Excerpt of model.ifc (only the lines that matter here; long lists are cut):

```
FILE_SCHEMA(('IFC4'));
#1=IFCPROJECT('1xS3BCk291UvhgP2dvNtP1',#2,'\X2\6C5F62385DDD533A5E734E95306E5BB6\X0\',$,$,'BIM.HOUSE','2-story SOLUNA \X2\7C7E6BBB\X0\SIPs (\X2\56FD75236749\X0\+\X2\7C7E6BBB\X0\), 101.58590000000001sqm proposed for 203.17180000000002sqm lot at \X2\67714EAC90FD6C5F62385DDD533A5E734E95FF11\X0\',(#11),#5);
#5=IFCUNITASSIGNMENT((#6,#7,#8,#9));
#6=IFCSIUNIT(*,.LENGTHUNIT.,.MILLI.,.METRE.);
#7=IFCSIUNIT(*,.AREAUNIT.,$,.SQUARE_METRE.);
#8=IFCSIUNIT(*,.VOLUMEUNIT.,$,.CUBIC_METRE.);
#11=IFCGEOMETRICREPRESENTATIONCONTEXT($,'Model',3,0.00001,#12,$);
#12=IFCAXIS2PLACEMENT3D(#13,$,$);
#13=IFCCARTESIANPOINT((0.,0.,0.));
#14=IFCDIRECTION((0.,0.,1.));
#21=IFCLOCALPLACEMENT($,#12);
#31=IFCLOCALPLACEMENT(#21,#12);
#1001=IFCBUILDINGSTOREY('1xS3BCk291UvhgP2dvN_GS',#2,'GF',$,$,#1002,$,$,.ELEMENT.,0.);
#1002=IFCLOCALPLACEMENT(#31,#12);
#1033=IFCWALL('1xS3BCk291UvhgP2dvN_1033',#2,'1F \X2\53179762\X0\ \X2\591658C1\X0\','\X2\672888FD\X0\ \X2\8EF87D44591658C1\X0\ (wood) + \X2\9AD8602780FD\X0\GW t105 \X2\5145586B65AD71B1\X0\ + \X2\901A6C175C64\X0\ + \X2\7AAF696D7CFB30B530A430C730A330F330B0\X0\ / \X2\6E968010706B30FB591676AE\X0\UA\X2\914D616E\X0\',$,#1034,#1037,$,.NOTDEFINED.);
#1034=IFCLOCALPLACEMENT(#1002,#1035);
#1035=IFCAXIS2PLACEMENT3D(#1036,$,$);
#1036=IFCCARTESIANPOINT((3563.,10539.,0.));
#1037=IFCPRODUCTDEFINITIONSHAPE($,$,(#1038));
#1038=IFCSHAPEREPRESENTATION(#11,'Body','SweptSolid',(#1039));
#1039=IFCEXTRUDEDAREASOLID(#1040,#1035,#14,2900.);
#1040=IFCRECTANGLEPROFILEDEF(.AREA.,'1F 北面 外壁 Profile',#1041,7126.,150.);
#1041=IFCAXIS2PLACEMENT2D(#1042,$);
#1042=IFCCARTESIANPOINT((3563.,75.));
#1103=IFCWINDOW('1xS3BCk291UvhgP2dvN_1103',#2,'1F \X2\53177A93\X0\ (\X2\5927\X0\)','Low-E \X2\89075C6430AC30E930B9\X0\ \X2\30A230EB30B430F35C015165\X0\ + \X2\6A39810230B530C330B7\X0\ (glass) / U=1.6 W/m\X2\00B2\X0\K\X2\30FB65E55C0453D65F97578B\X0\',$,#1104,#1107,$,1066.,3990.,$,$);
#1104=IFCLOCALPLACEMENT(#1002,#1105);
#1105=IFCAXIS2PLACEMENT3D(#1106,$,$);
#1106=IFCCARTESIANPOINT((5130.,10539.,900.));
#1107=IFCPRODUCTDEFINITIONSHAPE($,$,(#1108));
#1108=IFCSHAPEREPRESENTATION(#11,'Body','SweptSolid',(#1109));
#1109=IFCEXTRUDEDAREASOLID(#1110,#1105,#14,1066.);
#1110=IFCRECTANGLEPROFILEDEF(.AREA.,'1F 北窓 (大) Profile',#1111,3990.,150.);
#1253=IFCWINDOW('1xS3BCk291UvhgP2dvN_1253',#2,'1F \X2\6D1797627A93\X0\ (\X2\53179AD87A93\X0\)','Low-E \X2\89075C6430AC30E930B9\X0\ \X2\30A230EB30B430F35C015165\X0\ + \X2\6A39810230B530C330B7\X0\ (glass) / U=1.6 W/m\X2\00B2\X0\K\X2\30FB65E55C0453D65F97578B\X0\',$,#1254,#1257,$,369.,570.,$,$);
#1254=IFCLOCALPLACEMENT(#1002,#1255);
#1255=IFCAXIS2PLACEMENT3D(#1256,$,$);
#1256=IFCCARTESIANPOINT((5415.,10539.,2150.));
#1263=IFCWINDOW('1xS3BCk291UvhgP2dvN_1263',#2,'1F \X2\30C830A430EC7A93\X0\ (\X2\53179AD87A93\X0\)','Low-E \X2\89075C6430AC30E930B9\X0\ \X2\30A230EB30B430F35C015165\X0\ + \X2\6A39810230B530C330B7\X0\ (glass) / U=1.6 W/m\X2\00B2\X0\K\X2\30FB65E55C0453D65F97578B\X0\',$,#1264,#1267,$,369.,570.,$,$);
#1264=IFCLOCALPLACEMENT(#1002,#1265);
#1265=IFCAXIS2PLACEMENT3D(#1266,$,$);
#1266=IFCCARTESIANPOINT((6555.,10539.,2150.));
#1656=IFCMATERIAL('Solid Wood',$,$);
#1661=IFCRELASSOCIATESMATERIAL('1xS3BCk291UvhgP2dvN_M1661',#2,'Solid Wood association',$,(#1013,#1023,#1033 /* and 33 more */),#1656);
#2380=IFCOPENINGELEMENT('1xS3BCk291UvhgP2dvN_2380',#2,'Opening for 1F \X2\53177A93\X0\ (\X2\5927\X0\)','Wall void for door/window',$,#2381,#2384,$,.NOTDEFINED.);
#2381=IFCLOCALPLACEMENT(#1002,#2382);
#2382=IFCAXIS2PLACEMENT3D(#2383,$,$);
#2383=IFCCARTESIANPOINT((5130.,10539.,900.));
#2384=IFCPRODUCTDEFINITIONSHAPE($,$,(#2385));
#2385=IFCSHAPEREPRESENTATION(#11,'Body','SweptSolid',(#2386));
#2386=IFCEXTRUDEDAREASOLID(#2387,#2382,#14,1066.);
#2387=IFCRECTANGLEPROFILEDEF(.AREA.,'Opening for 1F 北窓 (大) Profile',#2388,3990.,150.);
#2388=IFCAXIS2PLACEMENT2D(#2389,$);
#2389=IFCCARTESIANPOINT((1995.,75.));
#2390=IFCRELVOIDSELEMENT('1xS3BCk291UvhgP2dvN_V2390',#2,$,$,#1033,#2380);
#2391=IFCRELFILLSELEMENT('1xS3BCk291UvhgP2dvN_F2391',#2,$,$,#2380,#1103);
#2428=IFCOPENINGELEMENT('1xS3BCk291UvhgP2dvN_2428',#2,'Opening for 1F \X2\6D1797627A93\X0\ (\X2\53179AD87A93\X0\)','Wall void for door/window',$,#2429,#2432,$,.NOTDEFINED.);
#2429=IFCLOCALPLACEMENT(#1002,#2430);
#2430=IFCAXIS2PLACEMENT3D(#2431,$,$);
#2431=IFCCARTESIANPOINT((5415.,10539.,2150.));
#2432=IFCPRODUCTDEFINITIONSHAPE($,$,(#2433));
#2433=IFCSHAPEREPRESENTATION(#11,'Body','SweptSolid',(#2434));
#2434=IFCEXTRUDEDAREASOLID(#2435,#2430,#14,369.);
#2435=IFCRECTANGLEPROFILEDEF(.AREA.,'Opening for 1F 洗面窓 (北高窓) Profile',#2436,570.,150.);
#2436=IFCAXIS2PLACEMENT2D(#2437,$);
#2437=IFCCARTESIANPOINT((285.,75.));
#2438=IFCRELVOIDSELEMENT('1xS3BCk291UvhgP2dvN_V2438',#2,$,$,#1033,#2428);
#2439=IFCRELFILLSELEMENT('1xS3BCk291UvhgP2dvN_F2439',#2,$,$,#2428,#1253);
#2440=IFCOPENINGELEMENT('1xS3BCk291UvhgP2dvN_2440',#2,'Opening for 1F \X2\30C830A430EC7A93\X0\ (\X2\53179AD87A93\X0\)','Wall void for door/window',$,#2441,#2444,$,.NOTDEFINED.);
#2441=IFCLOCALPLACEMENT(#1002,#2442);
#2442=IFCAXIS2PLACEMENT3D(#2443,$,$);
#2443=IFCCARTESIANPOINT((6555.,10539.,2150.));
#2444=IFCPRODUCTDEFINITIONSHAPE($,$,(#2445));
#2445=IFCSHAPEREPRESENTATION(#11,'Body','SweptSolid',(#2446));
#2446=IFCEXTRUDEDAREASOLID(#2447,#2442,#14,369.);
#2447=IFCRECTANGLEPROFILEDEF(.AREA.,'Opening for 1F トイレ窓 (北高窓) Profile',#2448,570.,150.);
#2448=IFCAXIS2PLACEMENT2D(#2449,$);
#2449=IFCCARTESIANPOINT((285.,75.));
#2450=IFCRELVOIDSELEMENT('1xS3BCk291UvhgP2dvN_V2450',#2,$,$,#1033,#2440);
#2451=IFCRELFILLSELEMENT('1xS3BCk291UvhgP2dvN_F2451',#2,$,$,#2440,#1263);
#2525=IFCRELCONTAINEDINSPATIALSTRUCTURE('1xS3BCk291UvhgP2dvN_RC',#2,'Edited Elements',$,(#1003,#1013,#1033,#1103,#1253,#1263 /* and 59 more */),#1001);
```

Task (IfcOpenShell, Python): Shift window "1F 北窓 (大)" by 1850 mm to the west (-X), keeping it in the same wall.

```python
import ifcopenshell
import ifcopenshell.api.geometry
import ifcopenshell.util.placement
import ifcopenshell.util.unit

model = ifcopenshell.open("model.ifc")
unit_scale = ifcopenshell.util.unit.calculate_unit_scale(model)

window = model.by_guid("1xS3BCk291UvhgP2dvN_1103")
opening = window.FillsVoids[0].RelatingOpeningElement
wall = opening.VoidsElements[0].RelatingBuildingElement

wall_matrix = ifcopenshell.util.placement.get_local_placement(wall.ObjectPlacement)
shift = wall_matrix[:3, 0] * -1.85 / unit_scale
before = ifcopenshell.util.placement.get_local_placement(window.ObjectPlacement)[:3, 3].copy()

# The window is not placed relative to its opening, so move both.
for product in (opening, window):
    matrix = ifcopenshell.util.placement.get_local_placement(product.ObjectPlacement)
    matrix[:3, 3] += shift
    ifcopenshell.api.geometry.edit_object_placement(model, product=product, matrix=matrix, is_si=False)

after = ifcopenshell.util.placement.get_local_placement(window.ObjectPlacement)[:3, 3]
print("window moved by", (after - before).round(3) + 0.0)

model.write("model_rev.ifc")
```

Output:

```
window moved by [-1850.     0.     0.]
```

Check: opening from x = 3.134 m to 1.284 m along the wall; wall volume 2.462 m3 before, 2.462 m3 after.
